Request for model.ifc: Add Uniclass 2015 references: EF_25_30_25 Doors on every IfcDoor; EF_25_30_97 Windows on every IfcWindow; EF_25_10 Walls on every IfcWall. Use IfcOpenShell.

First a look at what the model holds.

```python
import ifcopenshell

model = ifcopenshell.open("model.ifc")
print(model.schema)
print("classifications:", [c.Name for c in model.by_type("IfcClassification")])
for ifc_class in ("IfcDoor", "IfcRoof", "IfcStair", "IfcWall", "IfcWindow"):
    print(ifc_class, len(model.by_type(ifc_class)))
```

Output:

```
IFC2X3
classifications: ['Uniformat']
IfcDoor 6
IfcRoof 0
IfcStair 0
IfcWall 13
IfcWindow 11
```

```python
import ifcopenshell
import ifcopenshell.api.classification

model = ifcopenshell.open("model.ifc")

# IFC2X3 requires Source and Edition and has no link from the project to the system.
system = model.create_entity("IfcClassification", Source="NBS", Edition="2015", Name="Uniclass 2015")

codes = {
    "IfcDoor": ("EF_25_30_25", "Doors"),
    "IfcWindow": ("EF_25_30_97", "Windows"),
    "IfcWall": ("EF_25_10", "Walls"),
}
for ifc_class, (code, name) in codes.items():
    products = model.by_type(ifc_class)
    ifcopenshell.api.classification.add_reference(
        model, products=products, classification=system, identification=code, name=name
    )
    print(code, len(products))

model.write("model_edited.ifc")
```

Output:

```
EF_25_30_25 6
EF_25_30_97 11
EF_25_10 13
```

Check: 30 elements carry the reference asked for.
